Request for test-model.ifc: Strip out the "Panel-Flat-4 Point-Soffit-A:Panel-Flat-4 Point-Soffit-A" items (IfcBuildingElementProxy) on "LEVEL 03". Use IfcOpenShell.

First a look at what the model holds.

```python
import ifcopenshell
import ifcopenshell.util.element

model = ifcopenshell.open("test-model.ifc")
print(model.schema)
storey = next(s for s in model.by_type("IfcBuildingStorey") if s.Name == "LEVEL 03")
proxies = [e for e in ifcopenshell.util.element.get_decomposition(storey) if e.is_a("IfcBuildingElementProxy")]
seen = {}
for e in proxies:
    element_type = ifcopenshell.util.element.get_type(e)
    name = element_type.Name if element_type not in (None, e) else None
    seen[name] = seen.get(name, 0) + 1
for name, count in sorted(seen.items(), key=str):
    print(count, "x", name)
```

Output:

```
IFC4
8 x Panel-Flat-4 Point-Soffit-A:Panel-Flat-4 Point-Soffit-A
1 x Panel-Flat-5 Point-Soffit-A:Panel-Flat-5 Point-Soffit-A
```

```python
import ifcopenshell
import ifcopenshell.api.root
import ifcopenshell.util.element

model = ifcopenshell.open("test-model.ifc")

storey = next(s for s in model.by_type("IfcBuildingStorey") if s.Name == "LEVEL 03")
proxies = [e for e in ifcopenshell.util.element.get_decomposition(storey) if e.is_a("IfcBuildingElementProxy")]
targets = [e for e in proxies if (t := ifcopenshell.util.element.get_type(e)) not in (None, e) and t.Name == "Panel-Flat-4 Point-Soffit-A:Panel-Flat-4 Point-Soffit-A"]

for e in targets:
    ifcopenshell.api.root.remove_product(model, product=e)
print(len(targets), "removed")

model.write("test-model-out.ifc")
```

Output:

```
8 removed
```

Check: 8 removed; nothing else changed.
